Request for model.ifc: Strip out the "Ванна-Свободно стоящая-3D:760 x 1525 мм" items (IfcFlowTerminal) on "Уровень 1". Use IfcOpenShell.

First a look at what the model holds.

```python
import ifcopenshell
import ifcopenshell.util.element

model = ifcopenshell.open("model.ifc")
print(model.schema)
storey = next(s for s in model.by_type("IfcBuildingStorey") if s.Name == "Уровень 1")
terminals = [e for e in ifcopenshell.util.element.get_decomposition(storey) if e.is_a("IfcFlowTerminal")]
seen = {}
for e in terminals:
    element_type = ifcopenshell.util.element.get_type(e)
    name = element_type.Name if element_type not in (None, e) else None
    seen[name] = seen.get(name, 0) + 1
for name, count in sorted(seen.items(), key=str):
    print(count, "x", name)
```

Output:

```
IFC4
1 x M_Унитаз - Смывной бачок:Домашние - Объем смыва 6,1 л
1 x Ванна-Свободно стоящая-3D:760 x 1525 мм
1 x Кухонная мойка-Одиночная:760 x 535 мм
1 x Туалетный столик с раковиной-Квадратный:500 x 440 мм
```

```python
import ifcopenshell
import ifcopenshell.api.root
import ifcopenshell.util.element

model = ifcopenshell.open("model.ifc")

storey = next(s for s in model.by_type("IfcBuildingStorey") if s.Name == "Уровень 1")
terminals = [e for e in ifcopenshell.util.element.get_decomposition(storey) if e.is_a("IfcFlowTerminal")]
targets = [e for e in terminals if (t := ifcopenshell.util.element.get_type(e)) not in (None, e) and t.Name == "Ванна-Свободно стоящая-3D:760 x 1525 мм"]

for e in targets:
    ifcopenshell.api.root.remove_product(model, product=e)
print(len(targets), "removed")

model.write("model-out.ifc")
```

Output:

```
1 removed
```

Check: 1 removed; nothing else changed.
